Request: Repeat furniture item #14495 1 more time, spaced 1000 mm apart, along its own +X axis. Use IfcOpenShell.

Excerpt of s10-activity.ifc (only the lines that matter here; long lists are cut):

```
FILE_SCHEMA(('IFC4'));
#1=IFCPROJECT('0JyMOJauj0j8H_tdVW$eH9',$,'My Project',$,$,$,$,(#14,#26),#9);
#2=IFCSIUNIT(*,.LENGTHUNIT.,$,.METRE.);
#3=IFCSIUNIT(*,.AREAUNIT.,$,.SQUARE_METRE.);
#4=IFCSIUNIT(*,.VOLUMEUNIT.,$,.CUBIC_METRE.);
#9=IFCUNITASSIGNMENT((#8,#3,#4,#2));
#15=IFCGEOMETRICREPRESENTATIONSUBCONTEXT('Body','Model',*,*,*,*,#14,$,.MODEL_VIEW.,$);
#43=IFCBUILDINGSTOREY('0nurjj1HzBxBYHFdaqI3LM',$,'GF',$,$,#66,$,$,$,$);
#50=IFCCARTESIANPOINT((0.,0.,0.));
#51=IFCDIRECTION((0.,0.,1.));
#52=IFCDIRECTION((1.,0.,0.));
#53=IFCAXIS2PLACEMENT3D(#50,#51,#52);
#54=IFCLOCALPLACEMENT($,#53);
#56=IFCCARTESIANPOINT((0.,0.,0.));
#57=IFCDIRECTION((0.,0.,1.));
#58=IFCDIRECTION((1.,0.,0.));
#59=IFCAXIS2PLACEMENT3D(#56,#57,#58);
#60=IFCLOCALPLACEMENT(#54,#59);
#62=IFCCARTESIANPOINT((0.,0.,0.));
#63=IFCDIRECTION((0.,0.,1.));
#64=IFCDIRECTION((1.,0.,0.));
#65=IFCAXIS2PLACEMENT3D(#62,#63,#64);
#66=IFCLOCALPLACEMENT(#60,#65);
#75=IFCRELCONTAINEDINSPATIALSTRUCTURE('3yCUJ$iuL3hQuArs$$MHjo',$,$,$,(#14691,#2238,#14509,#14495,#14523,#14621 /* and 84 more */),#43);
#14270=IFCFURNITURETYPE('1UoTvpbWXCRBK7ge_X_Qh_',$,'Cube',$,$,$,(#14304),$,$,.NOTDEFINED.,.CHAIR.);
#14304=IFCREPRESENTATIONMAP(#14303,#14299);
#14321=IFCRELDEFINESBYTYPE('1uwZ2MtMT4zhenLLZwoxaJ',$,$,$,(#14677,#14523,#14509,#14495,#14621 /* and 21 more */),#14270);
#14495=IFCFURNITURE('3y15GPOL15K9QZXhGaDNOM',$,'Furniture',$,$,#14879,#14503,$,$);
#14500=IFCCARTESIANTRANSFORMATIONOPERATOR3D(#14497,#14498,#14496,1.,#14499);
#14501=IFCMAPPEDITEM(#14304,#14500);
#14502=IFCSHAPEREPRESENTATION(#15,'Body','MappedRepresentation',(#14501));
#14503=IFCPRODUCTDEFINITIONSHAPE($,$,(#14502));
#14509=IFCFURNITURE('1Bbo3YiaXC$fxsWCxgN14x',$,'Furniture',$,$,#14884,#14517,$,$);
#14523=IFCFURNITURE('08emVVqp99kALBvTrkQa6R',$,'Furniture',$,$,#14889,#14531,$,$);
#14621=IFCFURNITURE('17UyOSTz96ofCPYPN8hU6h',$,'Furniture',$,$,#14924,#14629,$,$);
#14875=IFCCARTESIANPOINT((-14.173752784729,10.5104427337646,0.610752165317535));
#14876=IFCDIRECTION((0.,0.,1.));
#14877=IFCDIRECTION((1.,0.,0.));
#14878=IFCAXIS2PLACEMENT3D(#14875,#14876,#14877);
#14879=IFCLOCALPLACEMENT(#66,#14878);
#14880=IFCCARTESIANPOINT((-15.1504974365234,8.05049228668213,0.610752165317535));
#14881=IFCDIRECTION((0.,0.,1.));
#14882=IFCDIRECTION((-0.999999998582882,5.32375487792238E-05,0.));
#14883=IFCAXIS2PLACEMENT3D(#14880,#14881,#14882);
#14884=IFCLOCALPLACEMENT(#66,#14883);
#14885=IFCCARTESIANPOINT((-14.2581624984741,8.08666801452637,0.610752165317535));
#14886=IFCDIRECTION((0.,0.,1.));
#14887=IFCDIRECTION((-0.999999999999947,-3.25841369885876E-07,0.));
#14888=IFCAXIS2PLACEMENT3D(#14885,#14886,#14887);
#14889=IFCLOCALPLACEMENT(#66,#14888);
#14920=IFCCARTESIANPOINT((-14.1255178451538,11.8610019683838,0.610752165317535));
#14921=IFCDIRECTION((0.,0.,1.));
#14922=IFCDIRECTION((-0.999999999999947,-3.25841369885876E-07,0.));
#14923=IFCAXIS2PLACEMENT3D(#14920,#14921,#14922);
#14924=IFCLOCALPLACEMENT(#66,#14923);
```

```python
import ifcopenshell
import ifcopenshell.api.geometry
import ifcopenshell.api.root
import ifcopenshell.util.element
import ifcopenshell.util.placement

model = ifcopenshell.open("s10-activity.ifc")

source = model.by_guid("3y15GPOL15K9QZXhGaDNOM")
base = ifcopenshell.util.placement.get_local_placement(source.ObjectPlacement)
step = base[:3, 0] * 1.0

for i in range(1, 2):
    copy = ifcopenshell.api.root.copy_class(model, product=source)
    copy.Representation = ifcopenshell.util.element.copy_deep(
        model, source.Representation, exclude=["IfcGeometricRepresentationContext", "IfcRepresentationMap"]
    )
    matrix = base.copy()
    matrix[:3, 3] += i * step
    print("added at", matrix[:3, 3].round(3) + 0.0)
    ifcopenshell.api.geometry.edit_object_placement(model, product=copy, matrix=matrix, is_si=False)

model.write("s10-activity_rev.ifc")
```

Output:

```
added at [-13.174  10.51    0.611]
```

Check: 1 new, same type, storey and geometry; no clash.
